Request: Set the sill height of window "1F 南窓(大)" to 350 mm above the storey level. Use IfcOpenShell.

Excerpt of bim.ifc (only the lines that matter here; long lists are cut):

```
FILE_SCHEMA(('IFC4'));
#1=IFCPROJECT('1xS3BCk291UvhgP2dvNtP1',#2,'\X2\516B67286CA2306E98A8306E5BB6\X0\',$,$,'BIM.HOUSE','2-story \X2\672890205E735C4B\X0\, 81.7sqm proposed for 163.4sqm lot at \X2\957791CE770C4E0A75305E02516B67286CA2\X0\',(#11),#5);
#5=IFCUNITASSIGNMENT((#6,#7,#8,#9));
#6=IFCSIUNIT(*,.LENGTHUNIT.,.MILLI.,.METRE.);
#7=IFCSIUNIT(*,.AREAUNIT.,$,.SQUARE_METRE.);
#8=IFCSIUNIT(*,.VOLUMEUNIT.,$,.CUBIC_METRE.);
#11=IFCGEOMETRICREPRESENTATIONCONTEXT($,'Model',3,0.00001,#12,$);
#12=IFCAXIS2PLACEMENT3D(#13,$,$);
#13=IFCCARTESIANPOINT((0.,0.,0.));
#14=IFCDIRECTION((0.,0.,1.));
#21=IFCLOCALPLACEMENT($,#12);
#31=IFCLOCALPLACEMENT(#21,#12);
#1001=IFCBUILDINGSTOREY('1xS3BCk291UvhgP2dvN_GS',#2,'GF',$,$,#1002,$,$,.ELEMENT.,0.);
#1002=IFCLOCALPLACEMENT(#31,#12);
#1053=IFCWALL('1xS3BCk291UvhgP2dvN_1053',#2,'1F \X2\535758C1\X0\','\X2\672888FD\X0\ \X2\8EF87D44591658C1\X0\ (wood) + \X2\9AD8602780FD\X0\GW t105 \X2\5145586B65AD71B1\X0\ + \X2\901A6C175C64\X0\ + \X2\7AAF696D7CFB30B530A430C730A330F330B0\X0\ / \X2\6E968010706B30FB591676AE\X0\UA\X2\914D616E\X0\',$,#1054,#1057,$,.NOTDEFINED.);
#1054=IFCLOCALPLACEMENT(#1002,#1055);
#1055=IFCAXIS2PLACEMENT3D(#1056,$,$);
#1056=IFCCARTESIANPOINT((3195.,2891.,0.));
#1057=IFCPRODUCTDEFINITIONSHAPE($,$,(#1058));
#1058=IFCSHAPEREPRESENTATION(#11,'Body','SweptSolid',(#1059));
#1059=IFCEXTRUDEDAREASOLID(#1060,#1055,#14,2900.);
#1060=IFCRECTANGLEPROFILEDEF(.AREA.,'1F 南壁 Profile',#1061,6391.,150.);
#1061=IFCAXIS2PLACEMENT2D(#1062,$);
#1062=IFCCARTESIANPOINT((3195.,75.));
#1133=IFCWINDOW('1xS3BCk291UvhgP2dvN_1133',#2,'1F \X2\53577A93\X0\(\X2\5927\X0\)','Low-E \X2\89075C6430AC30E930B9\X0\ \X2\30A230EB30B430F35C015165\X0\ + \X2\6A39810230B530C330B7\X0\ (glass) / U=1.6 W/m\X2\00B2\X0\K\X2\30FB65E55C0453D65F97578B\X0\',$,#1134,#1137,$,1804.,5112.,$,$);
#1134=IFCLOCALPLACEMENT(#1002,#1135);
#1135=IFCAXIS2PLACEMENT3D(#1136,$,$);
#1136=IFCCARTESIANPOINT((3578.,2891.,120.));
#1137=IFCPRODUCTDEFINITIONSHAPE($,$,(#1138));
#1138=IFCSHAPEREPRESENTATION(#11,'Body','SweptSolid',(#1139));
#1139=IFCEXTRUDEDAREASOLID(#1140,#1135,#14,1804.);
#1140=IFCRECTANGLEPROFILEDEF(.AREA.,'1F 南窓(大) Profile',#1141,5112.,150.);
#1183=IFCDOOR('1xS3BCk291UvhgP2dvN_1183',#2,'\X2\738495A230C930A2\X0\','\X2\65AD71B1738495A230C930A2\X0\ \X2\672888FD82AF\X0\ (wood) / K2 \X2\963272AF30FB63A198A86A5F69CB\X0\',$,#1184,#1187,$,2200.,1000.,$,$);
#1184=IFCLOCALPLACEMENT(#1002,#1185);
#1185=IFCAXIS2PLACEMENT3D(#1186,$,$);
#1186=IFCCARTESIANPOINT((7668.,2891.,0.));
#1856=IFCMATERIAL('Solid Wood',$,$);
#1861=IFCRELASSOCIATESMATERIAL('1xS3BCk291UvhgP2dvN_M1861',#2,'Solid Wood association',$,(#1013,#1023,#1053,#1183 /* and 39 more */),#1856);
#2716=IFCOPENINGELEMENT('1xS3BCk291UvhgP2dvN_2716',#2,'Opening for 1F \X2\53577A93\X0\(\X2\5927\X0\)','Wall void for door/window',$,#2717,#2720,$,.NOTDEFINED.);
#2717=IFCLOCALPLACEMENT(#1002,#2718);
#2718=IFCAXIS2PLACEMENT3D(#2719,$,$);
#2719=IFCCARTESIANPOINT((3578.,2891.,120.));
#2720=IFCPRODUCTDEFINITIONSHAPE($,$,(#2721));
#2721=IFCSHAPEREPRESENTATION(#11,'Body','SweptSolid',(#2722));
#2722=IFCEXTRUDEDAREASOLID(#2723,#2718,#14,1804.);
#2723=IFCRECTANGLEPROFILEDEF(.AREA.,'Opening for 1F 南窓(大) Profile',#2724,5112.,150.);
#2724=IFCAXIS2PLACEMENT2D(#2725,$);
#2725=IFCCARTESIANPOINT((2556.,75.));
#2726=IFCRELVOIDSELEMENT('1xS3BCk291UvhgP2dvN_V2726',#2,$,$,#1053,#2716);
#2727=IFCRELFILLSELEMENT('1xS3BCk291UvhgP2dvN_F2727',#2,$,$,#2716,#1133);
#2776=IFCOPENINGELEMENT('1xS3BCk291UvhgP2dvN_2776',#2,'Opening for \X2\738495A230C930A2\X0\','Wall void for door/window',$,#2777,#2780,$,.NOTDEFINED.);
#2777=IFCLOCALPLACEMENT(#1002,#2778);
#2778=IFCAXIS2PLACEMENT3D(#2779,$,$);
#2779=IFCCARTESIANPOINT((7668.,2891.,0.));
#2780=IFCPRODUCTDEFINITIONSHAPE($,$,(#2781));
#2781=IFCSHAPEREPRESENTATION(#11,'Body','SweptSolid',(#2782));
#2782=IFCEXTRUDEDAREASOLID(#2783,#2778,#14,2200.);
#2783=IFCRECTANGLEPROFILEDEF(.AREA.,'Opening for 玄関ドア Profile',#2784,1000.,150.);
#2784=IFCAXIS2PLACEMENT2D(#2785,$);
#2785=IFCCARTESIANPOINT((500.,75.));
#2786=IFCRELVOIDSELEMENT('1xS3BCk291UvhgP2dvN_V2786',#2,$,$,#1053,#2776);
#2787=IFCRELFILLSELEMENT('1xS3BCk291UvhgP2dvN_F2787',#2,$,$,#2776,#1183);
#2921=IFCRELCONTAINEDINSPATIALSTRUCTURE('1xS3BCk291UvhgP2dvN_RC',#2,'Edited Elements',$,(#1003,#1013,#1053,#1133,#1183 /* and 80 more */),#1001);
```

```python
import numpy as np
import ifcopenshell
import ifcopenshell.api.geometry
import ifcopenshell.geom
import ifcopenshell.util.element
import ifcopenshell.util.placement
import ifcopenshell.util.shape
import ifcopenshell.util.unit

model = ifcopenshell.open("bim.ifc")
unit_scale = ifcopenshell.util.unit.calculate_unit_scale(model)

window = model.by_id(1133)
opening = window.FillsVoids[0].RelatingOpeningElement
storey = ifcopenshell.util.element.get_container(window, ifc_class="IfcBuildingStorey")
level = ifcopenshell.util.placement.get_local_placement(storey.ObjectPlacement)[2, 3]

# The opening's origin need not be at the sill, so measure its lowest point.
shape = ifcopenshell.geom.create_shape(ifcopenshell.geom.settings(), opening)
bottom = ifcopenshell.util.shape.get_shape_bottom_elevation(shape, shape.geometry) / unit_scale
dz = level + 0.35 / unit_scale - bottom

shift = np.array([0.0, 0.0, dz])
# The window is not placed relative to its opening, so move both.
for product in (opening, window):
    matrix = ifcopenshell.util.placement.get_local_placement(product.ObjectPlacement)
    matrix[:3, 3] += shift
    ifcopenshell.api.geometry.edit_object_placement(model, product=product, matrix=matrix, is_si=False)

print(f"moved by {dz * unit_scale:+.3f} m")

model.write("bim_edited.ifc")
```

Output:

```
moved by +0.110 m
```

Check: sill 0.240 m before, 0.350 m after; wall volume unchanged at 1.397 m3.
